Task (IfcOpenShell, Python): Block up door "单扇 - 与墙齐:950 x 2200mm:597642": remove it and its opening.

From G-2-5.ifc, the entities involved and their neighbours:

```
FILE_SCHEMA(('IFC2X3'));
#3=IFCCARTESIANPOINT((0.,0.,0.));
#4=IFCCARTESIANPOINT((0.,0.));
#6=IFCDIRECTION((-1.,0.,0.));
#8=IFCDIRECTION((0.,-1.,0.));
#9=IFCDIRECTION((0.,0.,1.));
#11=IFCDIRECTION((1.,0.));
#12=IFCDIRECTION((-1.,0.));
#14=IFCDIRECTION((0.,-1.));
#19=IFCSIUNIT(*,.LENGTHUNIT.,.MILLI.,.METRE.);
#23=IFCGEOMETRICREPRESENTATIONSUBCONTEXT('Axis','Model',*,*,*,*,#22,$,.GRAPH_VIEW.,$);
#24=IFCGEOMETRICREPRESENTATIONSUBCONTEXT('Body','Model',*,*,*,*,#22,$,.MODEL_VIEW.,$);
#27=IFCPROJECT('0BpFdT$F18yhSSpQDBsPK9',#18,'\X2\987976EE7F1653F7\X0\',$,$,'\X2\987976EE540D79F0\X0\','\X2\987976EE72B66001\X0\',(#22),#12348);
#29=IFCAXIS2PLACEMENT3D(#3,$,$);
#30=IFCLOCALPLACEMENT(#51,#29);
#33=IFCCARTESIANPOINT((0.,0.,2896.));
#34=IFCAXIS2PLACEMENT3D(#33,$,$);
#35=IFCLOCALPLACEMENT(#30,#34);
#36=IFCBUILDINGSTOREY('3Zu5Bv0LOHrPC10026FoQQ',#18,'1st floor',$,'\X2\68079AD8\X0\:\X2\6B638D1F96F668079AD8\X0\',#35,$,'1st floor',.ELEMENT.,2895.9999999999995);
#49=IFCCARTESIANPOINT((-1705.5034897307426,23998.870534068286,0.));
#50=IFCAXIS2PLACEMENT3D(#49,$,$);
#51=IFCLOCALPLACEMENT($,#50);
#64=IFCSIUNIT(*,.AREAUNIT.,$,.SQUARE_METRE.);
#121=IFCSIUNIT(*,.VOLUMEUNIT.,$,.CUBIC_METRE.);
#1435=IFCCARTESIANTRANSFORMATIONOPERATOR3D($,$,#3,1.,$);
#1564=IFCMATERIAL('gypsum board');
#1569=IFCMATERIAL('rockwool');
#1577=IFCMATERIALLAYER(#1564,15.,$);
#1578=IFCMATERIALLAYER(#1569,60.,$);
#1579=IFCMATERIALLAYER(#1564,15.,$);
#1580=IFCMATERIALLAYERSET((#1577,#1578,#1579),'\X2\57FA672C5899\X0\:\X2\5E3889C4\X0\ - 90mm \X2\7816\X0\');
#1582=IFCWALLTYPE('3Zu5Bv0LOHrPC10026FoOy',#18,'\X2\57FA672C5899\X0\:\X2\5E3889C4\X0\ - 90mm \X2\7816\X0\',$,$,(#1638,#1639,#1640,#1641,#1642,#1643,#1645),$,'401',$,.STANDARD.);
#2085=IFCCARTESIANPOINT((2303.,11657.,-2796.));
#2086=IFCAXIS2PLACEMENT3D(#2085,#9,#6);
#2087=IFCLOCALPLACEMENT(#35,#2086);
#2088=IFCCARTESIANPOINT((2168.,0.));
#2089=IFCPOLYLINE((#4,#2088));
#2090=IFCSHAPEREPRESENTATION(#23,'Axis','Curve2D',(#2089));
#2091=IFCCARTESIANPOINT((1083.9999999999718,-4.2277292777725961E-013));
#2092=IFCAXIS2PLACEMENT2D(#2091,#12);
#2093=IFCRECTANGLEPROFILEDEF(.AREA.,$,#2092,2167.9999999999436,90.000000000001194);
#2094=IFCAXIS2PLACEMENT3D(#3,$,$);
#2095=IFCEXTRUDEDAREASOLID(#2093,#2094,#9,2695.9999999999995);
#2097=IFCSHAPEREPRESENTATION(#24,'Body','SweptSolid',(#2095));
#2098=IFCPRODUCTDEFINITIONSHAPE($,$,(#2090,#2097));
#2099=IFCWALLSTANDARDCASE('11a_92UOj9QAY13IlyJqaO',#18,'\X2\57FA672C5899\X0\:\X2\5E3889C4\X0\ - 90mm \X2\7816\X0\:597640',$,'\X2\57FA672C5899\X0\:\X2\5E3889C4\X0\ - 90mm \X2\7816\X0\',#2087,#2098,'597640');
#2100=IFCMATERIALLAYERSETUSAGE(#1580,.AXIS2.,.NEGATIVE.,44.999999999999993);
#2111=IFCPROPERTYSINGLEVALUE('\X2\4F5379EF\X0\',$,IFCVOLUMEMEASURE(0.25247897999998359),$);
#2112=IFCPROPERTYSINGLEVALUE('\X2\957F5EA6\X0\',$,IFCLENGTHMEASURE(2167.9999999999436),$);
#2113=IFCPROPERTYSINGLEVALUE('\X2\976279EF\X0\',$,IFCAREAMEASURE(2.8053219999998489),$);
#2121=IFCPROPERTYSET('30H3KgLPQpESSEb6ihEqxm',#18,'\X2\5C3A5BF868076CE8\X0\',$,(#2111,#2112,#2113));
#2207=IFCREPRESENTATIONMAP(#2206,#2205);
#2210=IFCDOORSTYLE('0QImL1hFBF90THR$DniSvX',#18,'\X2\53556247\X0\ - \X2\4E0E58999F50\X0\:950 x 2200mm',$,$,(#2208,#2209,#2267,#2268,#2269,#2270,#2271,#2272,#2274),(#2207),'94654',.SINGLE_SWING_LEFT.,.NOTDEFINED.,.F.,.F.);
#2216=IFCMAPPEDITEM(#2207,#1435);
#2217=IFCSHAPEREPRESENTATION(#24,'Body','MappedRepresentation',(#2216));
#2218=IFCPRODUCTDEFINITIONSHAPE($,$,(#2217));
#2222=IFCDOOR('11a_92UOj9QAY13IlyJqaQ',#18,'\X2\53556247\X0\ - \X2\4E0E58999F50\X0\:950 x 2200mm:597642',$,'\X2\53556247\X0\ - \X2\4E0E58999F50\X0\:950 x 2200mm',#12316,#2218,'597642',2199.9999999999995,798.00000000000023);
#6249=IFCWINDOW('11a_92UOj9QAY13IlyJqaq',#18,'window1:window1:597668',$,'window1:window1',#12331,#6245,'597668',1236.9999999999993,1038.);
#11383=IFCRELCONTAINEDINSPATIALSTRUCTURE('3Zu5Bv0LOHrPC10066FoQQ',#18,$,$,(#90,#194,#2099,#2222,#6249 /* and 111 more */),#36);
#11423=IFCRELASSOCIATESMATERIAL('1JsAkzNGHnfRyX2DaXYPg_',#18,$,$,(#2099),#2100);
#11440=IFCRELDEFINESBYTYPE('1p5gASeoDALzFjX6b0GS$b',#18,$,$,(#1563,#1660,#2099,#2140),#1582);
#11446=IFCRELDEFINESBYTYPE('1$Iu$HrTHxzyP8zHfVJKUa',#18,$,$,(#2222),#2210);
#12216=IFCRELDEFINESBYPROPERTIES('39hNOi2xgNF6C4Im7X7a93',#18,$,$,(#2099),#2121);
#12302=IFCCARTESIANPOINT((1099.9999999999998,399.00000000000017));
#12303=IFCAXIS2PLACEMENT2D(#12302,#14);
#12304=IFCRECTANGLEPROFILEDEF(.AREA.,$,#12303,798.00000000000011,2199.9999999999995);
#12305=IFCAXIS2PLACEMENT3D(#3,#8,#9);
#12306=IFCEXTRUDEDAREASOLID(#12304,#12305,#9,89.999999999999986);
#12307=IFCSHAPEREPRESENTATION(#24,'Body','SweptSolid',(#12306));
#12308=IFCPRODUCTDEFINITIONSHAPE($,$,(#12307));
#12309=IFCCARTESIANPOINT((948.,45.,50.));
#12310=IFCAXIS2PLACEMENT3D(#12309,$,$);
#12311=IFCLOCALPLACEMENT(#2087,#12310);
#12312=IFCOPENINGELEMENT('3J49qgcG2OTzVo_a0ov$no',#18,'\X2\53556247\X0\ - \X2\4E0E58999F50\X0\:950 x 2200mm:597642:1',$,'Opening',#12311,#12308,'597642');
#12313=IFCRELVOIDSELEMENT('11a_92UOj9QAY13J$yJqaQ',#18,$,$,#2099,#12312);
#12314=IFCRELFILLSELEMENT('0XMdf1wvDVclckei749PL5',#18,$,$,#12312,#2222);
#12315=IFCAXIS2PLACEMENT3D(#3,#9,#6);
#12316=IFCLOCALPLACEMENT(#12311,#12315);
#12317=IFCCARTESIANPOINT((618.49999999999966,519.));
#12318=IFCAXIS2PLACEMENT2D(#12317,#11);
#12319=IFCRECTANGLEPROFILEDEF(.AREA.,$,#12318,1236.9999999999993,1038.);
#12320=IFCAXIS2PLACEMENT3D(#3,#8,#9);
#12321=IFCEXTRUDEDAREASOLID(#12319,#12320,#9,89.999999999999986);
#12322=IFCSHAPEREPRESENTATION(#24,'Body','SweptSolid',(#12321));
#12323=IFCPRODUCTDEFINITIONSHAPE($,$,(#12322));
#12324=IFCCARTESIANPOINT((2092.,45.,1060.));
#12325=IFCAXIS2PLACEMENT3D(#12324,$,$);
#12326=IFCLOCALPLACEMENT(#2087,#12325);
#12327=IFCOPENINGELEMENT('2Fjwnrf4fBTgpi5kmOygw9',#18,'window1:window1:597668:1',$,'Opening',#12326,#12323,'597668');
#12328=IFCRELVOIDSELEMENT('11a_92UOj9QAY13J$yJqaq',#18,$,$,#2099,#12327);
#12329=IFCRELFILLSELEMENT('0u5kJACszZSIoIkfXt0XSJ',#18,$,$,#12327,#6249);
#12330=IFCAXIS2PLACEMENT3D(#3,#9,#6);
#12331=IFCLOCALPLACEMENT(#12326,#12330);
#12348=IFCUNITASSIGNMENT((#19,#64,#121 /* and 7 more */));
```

```python
import ifcopenshell
import ifcopenshell.api.feature
import ifcopenshell.api.pset
import ifcopenshell.api.root
import ifcopenshell.geom
import ifcopenshell.util.element
import ifcopenshell.util.shape
import ifcopenshell.util.unit

model = ifcopenshell.open("G-2-5.ifc")
area_scale = ifcopenshell.util.unit.calculate_unit_scale(model, "AREAUNIT")
volume_scale = ifcopenshell.util.unit.calculate_unit_scale(model, "VOLUMEUNIT")
settings = ifcopenshell.geom.settings()


def volume(element):
    """Net volume in cubic metres, openings subtracted."""
    shape = ifcopenshell.geom.create_shape(settings, element)
    return ifcopenshell.util.shape.get_volume(shape.geometry)


door = model.by_guid("11a_92UOj9QAY13IlyJqaQ")
opening = door.FillsVoids[0].RelatingOpeningElement
wall = opening.VoidsElements[0].RelatingBuildingElement
before = volume(wall)

ifcopenshell.api.root.remove_product(model, product=door)
ifcopenshell.api.feature.remove_feature(model, feature=opening)

after = volume(wall)
thickness = 0.09  # wall thickness in metres

# Update the wall's stored quantities.
pset = model.by_id(ifcopenshell.util.element.get_pset(wall, "尺寸标注", should_inherit=False)["id"])
ifcopenshell.api.pset.edit_pset(model, pset=pset, properties={
    "体积": model.create_entity("IfcVolumeMeasure", after / volume_scale),
    "面积": model.create_entity("IfcAreaMeasure", after / thickness / area_scale),
})

print(f"wall volume {before:.3f} -> {after:.3f} m3")

model.write("G-2-5_v2.ifc")
```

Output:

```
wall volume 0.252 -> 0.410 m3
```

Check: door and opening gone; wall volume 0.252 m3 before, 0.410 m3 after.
